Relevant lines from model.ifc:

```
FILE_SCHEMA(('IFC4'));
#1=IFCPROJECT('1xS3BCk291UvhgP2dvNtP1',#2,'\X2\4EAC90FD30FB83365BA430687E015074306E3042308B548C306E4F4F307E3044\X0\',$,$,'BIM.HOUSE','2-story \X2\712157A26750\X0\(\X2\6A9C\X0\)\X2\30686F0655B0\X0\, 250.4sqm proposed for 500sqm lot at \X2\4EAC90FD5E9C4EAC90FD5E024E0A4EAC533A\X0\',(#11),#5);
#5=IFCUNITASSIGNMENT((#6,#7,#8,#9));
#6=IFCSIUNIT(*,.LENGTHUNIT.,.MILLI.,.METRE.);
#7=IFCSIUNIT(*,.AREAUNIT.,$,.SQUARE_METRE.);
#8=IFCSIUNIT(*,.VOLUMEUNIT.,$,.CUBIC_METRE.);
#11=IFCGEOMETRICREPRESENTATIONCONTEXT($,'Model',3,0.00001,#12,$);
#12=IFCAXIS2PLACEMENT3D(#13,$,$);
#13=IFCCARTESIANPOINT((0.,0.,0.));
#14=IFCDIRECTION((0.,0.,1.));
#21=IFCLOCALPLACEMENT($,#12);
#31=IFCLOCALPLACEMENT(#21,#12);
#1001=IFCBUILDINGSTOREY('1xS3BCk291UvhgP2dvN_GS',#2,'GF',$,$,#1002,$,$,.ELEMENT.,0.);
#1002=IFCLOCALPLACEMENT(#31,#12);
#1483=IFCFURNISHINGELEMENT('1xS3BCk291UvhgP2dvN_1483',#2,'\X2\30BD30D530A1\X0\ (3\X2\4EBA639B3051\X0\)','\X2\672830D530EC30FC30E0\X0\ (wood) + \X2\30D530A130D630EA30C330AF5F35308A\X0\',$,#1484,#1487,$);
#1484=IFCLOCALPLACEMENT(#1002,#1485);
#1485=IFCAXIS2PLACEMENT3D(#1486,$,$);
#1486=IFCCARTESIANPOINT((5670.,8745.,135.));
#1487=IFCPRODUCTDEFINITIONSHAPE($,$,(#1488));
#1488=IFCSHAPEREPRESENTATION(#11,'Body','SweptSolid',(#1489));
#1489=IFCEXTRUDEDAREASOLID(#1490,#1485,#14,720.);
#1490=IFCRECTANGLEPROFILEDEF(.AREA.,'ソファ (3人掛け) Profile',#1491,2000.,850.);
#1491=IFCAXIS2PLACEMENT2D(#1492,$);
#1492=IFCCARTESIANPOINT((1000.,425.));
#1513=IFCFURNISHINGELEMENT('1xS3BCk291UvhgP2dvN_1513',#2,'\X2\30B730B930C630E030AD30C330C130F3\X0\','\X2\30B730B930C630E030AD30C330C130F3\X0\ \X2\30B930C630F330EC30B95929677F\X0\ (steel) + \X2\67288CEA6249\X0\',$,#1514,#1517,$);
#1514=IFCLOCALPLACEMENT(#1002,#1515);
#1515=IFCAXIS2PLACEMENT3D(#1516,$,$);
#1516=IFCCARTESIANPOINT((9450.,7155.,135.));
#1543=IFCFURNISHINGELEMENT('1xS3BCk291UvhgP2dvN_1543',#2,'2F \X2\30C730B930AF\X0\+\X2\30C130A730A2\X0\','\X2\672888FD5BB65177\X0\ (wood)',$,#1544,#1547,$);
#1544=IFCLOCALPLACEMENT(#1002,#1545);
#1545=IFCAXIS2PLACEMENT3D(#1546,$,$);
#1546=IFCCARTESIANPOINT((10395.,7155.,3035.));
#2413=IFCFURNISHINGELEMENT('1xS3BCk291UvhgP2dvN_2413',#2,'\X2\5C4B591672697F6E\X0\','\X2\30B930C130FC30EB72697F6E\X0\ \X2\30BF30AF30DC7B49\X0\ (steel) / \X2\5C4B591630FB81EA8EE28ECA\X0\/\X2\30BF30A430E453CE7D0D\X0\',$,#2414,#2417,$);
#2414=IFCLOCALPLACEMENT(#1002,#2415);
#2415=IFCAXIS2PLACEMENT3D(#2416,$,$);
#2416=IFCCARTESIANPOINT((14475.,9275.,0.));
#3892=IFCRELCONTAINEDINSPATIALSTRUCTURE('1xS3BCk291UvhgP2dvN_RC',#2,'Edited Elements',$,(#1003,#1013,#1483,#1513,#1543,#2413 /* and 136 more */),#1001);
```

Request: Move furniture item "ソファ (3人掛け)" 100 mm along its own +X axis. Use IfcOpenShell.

```python
import ifcopenshell
import ifcopenshell.api.geometry
import ifcopenshell.util.placement
import ifcopenshell.util.unit

model = ifcopenshell.open("model.ifc")
unit_scale = ifcopenshell.util.unit.calculate_unit_scale(model)

item = model.by_guid("1xS3BCk291UvhgP2dvN_1483")
matrix = ifcopenshell.util.placement.get_local_placement(item.ObjectPlacement)
matrix[:3, 3] += matrix[:3, 0] * 0.1 / unit_scale
ifcopenshell.api.geometry.edit_object_placement(model, product=item, matrix=matrix, is_si=False)

print(ifcopenshell.util.placement.get_local_placement(item.ObjectPlacement).round(3) + 0.0)

model.write("model_rev.ifc")
```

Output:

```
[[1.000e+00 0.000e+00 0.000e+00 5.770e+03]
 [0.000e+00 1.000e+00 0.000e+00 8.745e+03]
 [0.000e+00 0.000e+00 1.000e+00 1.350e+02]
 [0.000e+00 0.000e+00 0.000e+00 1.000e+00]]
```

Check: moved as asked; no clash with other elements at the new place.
